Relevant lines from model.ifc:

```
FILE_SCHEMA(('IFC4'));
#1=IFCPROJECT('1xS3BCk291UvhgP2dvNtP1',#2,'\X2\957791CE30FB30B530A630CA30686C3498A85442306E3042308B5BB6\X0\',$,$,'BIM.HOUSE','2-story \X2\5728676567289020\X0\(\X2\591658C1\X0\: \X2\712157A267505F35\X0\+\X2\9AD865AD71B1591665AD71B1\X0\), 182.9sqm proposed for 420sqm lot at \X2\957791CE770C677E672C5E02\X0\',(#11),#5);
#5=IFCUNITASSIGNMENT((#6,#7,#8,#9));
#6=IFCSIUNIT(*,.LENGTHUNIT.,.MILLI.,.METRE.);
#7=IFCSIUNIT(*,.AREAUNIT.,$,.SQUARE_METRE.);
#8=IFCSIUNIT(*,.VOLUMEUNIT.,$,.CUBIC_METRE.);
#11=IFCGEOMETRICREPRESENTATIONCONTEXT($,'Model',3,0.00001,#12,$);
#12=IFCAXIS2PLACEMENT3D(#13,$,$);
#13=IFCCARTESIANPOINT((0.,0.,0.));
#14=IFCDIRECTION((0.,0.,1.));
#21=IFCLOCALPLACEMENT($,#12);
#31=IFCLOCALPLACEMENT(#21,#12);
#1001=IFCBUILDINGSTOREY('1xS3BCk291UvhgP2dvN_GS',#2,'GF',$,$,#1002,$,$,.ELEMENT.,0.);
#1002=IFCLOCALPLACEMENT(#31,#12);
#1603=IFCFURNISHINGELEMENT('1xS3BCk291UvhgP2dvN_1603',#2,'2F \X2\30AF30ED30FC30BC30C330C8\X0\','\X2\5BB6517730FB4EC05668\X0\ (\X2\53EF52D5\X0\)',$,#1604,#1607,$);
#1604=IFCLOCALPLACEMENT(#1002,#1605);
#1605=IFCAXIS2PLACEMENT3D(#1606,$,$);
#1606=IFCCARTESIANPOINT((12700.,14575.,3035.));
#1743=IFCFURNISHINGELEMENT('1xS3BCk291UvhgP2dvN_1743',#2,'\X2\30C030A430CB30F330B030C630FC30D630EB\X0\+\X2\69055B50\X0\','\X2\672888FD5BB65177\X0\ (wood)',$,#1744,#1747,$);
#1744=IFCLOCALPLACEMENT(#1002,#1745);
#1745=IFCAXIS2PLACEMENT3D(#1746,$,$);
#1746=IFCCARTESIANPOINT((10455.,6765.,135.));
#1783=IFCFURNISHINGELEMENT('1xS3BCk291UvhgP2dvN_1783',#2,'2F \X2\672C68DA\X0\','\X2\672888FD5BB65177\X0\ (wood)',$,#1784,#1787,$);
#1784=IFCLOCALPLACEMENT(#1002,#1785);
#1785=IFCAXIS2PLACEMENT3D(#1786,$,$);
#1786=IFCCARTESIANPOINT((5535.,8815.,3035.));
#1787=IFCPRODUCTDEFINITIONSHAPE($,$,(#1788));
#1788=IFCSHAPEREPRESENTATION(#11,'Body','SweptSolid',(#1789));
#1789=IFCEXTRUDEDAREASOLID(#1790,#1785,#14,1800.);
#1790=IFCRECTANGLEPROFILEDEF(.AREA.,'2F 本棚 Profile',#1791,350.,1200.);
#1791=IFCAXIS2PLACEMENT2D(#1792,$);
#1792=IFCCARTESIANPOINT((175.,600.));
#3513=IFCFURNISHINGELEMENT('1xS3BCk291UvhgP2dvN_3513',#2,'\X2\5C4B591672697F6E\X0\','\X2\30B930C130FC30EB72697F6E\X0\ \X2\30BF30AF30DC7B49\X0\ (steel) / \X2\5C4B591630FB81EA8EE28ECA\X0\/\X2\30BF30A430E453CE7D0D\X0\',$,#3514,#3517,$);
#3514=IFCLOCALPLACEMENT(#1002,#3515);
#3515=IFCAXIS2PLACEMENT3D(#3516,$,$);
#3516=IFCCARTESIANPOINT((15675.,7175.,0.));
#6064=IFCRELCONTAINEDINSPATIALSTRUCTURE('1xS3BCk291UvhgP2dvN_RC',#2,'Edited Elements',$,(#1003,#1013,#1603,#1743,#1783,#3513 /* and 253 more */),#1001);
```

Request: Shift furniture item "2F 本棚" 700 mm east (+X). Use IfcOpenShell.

```python
import ifcopenshell
import ifcopenshell.api.geometry
import ifcopenshell.util.placement

model = ifcopenshell.open("model.ifc")

item = model.by_guid("1xS3BCk291UvhgP2dvN_1783")
matrix = ifcopenshell.util.placement.get_local_placement(item.ObjectPlacement)
matrix[0, 3] += 700.0
ifcopenshell.api.geometry.edit_object_placement(model, product=item, matrix=matrix, is_si=False)

print(ifcopenshell.util.placement.get_local_placement(item.ObjectPlacement).round(3) + 0.0)

model.write("model-out.ifc")
```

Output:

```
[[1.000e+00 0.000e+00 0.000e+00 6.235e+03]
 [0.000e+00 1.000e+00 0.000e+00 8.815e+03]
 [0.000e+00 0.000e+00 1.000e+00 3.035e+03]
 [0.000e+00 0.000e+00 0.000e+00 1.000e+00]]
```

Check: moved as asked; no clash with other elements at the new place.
